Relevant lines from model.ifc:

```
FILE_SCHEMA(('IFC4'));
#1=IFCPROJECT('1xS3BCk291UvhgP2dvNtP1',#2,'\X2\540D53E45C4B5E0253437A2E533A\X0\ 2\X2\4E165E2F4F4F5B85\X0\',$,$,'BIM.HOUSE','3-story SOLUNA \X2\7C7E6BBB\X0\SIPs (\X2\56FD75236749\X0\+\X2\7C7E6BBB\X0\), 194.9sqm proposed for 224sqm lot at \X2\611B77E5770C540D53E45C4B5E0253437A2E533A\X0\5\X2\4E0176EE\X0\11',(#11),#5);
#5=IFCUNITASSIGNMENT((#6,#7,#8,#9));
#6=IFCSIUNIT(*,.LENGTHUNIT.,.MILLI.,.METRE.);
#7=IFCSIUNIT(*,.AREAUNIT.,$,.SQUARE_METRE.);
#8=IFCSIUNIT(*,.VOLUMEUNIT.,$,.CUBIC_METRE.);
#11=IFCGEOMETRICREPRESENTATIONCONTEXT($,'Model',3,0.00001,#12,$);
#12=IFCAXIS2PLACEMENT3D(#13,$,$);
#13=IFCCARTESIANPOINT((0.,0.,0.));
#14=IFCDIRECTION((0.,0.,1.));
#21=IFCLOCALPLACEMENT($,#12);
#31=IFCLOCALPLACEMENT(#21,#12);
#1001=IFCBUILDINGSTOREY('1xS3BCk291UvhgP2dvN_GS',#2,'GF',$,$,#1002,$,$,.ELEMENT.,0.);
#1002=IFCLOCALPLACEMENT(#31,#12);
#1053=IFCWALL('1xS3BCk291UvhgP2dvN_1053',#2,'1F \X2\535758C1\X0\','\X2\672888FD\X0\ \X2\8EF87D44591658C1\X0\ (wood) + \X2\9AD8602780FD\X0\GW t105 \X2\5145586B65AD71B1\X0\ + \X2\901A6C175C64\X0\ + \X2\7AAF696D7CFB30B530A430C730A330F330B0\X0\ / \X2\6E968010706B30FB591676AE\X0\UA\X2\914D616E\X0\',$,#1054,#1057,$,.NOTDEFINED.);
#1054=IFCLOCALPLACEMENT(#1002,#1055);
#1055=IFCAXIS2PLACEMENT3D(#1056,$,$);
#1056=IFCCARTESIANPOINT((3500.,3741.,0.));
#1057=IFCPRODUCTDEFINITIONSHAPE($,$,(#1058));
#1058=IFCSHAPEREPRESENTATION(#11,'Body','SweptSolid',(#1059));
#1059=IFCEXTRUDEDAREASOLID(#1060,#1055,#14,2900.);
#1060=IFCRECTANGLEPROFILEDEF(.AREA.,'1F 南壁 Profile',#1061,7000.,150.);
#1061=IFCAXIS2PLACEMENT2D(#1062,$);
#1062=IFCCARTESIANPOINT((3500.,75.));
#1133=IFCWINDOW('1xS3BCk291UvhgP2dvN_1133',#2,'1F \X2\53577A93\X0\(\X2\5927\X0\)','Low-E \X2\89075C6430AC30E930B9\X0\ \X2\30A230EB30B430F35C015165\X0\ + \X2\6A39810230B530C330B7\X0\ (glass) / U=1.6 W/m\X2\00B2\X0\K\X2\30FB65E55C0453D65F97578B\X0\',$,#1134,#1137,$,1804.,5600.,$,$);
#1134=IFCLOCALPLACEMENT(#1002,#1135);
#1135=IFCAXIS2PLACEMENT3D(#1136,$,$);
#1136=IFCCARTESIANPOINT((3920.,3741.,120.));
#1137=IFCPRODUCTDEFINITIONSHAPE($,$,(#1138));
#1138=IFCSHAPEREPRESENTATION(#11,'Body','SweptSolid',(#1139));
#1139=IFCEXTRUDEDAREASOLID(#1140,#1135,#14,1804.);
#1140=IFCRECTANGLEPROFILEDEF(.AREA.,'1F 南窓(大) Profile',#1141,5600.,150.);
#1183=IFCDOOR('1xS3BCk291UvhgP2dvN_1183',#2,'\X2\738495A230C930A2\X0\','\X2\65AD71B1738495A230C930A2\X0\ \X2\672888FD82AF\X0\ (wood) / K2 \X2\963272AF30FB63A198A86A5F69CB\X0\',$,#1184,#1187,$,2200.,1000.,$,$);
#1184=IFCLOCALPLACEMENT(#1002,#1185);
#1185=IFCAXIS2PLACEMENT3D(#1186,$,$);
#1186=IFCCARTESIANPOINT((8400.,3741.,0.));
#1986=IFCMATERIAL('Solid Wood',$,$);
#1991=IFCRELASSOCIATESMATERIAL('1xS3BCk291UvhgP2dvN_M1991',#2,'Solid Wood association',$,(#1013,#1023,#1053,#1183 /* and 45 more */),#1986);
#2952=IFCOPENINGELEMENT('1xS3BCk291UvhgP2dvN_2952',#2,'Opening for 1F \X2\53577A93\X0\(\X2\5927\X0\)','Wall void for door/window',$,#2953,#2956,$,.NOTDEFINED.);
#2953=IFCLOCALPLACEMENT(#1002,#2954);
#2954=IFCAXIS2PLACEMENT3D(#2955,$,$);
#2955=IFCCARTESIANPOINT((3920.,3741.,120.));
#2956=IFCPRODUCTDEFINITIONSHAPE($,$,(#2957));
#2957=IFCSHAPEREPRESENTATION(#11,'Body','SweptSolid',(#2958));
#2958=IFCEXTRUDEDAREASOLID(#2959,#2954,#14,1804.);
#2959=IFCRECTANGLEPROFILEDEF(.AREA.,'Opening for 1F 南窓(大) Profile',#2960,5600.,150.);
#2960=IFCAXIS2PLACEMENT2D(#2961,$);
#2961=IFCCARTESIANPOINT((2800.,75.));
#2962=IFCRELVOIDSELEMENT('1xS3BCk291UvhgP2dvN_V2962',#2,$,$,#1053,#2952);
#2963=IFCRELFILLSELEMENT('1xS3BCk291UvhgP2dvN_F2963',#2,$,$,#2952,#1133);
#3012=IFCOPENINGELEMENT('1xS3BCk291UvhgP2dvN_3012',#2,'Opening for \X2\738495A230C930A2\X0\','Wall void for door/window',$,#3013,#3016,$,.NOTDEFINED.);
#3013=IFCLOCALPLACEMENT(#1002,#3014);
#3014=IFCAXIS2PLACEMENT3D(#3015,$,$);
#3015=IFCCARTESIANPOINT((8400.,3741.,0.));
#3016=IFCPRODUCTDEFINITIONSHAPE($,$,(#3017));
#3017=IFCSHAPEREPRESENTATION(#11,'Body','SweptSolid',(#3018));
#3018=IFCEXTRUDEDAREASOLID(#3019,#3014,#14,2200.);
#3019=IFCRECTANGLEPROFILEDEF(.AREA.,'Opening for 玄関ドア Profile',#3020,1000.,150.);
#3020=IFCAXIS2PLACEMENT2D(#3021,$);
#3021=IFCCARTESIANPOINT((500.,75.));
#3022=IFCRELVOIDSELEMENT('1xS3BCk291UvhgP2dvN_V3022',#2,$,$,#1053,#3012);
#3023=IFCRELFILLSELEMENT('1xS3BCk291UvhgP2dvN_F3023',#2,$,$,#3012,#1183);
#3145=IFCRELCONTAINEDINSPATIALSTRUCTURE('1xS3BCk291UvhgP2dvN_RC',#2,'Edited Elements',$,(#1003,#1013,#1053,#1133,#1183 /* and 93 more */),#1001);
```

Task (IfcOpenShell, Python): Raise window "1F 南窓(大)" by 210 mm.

```python
import numpy as np
import ifcopenshell
import ifcopenshell.api.geometry
import ifcopenshell.util.placement
import ifcopenshell.util.unit

model = ifcopenshell.open("model.ifc")
unit_scale = ifcopenshell.util.unit.calculate_unit_scale(model)

window = model.by_guid("1xS3BCk291UvhgP2dvN_1133")
opening = window.FillsVoids[0].RelatingOpeningElement
dz = 210.0

shift = np.array([0.0, 0.0, dz])
# The window is not placed relative to its opening, so move both.
for product in (opening, window):
    matrix = ifcopenshell.util.placement.get_local_placement(product.ObjectPlacement)
    matrix[:3, 3] += shift
    ifcopenshell.api.geometry.edit_object_placement(model, product=product, matrix=matrix, is_si=False)

print(f"moved by {dz * unit_scale:+.3f} m")

model.write("model_v2.ifc")
```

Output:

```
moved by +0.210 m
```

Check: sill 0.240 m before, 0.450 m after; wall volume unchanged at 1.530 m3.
